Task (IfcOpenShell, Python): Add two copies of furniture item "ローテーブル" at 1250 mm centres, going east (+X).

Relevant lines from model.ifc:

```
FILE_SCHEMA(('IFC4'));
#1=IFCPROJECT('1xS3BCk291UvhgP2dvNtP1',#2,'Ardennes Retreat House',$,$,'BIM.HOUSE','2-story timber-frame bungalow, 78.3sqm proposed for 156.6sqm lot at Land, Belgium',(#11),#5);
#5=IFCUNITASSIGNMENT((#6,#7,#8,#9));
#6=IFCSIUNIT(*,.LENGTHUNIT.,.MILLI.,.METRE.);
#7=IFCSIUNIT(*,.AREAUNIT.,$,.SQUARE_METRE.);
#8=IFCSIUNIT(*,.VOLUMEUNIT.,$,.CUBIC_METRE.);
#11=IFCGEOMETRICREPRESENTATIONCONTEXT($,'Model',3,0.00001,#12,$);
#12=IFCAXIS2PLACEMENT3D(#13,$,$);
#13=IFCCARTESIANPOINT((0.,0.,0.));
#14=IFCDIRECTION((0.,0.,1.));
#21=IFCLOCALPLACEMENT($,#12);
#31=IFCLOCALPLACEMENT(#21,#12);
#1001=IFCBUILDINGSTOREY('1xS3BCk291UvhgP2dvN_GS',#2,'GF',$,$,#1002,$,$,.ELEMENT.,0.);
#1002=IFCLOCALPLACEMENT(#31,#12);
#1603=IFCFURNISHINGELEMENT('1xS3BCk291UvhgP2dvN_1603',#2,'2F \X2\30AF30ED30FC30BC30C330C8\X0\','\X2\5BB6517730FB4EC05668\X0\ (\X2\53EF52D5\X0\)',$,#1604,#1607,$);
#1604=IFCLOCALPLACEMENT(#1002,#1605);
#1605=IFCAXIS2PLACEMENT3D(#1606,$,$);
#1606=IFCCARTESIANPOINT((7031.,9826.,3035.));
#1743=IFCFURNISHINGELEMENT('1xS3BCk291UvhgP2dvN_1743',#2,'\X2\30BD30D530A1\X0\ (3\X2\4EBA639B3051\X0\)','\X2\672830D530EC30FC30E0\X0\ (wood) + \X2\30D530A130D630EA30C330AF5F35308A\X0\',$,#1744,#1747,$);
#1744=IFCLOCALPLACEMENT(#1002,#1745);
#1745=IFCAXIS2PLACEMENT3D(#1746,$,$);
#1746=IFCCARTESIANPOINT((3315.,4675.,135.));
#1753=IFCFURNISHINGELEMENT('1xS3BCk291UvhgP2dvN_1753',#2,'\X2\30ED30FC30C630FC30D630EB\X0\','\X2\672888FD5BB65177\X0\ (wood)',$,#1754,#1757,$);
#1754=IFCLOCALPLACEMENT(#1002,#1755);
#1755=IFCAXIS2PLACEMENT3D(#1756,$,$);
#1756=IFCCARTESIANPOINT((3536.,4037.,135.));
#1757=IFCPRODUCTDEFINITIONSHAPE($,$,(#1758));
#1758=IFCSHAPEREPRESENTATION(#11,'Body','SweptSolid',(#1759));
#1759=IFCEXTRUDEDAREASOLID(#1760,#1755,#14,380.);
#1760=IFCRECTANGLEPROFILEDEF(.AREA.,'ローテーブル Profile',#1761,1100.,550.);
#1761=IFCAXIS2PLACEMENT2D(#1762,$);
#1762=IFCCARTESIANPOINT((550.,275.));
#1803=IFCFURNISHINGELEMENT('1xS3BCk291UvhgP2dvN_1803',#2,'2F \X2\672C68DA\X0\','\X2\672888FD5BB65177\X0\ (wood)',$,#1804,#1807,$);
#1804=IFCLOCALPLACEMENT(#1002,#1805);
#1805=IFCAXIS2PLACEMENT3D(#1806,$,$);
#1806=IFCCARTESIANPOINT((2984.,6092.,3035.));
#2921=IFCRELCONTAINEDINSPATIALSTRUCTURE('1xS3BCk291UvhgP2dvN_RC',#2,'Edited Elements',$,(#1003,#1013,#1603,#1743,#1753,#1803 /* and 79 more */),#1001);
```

```python
import numpy as np
import ifcopenshell
import ifcopenshell.api.geometry
import ifcopenshell.api.root
import ifcopenshell.util.element
import ifcopenshell.util.placement

model = ifcopenshell.open("model.ifc")


def reuse_history(source, copy):
    """copy_class also copies each property set's owner history, people and application; keep the originals."""
    for rel in copy.IsDefinedBy:
        if rel.is_a("IfcRelDefinesByProperties") and (history := rel.RelatingPropertyDefinition.OwnerHistory):
            rel.RelatingPropertyDefinition.OwnerHistory = source.OwnerHistory
            ifcopenshell.util.element.remove_deep2(model, history)


source = model.by_guid("1xS3BCk291UvhgP2dvN_1753")
base = ifcopenshell.util.placement.get_local_placement(source.ObjectPlacement)
step = np.array([1.0, 0.0, 0.0]) * 1250.0

for i in range(1, 3):
    copy = ifcopenshell.api.root.copy_class(model, product=source)
    copy.Representation = ifcopenshell.util.element.copy_deep(
        model, source.Representation, exclude=["IfcGeometricRepresentationContext", "IfcRepresentationMap"]
    )
    reuse_history(source, copy)
    matrix = base.copy()
    matrix[:3, 3] += i * step
    print("added at", matrix[:3, 3].round(3) + 0.0)
    ifcopenshell.api.geometry.edit_object_placement(model, product=copy, matrix=matrix, is_si=False)

model.write("model_updated.ifc")
```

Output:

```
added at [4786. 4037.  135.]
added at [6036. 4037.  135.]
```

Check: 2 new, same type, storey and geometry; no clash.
